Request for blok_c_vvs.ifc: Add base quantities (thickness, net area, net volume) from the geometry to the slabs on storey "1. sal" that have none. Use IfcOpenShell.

First a look at what the model holds.

```python
import ifcopenshell
import ifcopenshell.util.element
import ifcopenshell.util.unit

model = ifcopenshell.open("blok_c_vvs.ifc")
print(model.schema)
for unit_type in ("LENGTHUNIT", "AREAUNIT", "VOLUMEUNIT"):
    print(unit_type, ifcopenshell.util.unit.calculate_unit_scale(model, unit_type))
storey = next(s for s in model.by_type("IfcBuildingStorey") if s.Name == "1. sal")
slabs = [e for e in ifcopenshell.util.element.get_decomposition(storey) if e.is_a("IfcSlab")]
for e in sorted(slabs, key=lambda e: e.id()):
    print(e.id(), e.is_a(), e.Name, list(ifcopenshell.util.element.get_psets(e, qtos_only=True)), sep=" | ")
```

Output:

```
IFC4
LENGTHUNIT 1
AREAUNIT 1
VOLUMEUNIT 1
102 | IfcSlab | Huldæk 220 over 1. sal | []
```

```python
import ifcopenshell
import ifcopenshell.api.pset
import ifcopenshell.geom
import ifcopenshell.util.element
import ifcopenshell.util.shape
import ifcopenshell.util.unit

model = ifcopenshell.open("blok_c_vvs.ifc")
unit_scale = ifcopenshell.util.unit.calculate_unit_scale(model)
area_scale = ifcopenshell.util.unit.calculate_unit_scale(model, "AREAUNIT")
volume_scale = ifcopenshell.util.unit.calculate_unit_scale(model, "VOLUMEUNIT")
settings = ifcopenshell.geom.settings()

storey = next(s for s in model.by_type("IfcBuildingStorey") if s.Name == "1. sal")
slabs = [e for e in ifcopenshell.util.element.get_decomposition(storey) if e.is_a("IfcSlab")]

for e in sorted(slabs, key=lambda e: e.id()):
    if ifcopenshell.util.element.get_psets(e, qtos_only=True, should_inherit=False):
        continue
    # Geometry comes back in metres, in the element's own axes.
    shape = ifcopenshell.geom.create_shape(settings, e)
    values = {
        "Width": ifcopenshell.util.shape.get_z(shape.geometry) / unit_scale,
        "NetArea": ifcopenshell.util.shape.get_footprint_area(shape.geometry) / area_scale,
        "NetVolume": ifcopenshell.util.shape.get_volume(shape.geometry) / volume_scale,
    }
    qto = ifcopenshell.api.pset.add_qto(model, product=e, name="Qto_SlabBaseQuantities")
    ifcopenshell.api.pset.edit_qto(model, qto=qto, properties=values)
    print(e.id(), {k: round(v, 3) for k, v in values.items()})

model.write("blok_c_vvs_edited.ifc")
```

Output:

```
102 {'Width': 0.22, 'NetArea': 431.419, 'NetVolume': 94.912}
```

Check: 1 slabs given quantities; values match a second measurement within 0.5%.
